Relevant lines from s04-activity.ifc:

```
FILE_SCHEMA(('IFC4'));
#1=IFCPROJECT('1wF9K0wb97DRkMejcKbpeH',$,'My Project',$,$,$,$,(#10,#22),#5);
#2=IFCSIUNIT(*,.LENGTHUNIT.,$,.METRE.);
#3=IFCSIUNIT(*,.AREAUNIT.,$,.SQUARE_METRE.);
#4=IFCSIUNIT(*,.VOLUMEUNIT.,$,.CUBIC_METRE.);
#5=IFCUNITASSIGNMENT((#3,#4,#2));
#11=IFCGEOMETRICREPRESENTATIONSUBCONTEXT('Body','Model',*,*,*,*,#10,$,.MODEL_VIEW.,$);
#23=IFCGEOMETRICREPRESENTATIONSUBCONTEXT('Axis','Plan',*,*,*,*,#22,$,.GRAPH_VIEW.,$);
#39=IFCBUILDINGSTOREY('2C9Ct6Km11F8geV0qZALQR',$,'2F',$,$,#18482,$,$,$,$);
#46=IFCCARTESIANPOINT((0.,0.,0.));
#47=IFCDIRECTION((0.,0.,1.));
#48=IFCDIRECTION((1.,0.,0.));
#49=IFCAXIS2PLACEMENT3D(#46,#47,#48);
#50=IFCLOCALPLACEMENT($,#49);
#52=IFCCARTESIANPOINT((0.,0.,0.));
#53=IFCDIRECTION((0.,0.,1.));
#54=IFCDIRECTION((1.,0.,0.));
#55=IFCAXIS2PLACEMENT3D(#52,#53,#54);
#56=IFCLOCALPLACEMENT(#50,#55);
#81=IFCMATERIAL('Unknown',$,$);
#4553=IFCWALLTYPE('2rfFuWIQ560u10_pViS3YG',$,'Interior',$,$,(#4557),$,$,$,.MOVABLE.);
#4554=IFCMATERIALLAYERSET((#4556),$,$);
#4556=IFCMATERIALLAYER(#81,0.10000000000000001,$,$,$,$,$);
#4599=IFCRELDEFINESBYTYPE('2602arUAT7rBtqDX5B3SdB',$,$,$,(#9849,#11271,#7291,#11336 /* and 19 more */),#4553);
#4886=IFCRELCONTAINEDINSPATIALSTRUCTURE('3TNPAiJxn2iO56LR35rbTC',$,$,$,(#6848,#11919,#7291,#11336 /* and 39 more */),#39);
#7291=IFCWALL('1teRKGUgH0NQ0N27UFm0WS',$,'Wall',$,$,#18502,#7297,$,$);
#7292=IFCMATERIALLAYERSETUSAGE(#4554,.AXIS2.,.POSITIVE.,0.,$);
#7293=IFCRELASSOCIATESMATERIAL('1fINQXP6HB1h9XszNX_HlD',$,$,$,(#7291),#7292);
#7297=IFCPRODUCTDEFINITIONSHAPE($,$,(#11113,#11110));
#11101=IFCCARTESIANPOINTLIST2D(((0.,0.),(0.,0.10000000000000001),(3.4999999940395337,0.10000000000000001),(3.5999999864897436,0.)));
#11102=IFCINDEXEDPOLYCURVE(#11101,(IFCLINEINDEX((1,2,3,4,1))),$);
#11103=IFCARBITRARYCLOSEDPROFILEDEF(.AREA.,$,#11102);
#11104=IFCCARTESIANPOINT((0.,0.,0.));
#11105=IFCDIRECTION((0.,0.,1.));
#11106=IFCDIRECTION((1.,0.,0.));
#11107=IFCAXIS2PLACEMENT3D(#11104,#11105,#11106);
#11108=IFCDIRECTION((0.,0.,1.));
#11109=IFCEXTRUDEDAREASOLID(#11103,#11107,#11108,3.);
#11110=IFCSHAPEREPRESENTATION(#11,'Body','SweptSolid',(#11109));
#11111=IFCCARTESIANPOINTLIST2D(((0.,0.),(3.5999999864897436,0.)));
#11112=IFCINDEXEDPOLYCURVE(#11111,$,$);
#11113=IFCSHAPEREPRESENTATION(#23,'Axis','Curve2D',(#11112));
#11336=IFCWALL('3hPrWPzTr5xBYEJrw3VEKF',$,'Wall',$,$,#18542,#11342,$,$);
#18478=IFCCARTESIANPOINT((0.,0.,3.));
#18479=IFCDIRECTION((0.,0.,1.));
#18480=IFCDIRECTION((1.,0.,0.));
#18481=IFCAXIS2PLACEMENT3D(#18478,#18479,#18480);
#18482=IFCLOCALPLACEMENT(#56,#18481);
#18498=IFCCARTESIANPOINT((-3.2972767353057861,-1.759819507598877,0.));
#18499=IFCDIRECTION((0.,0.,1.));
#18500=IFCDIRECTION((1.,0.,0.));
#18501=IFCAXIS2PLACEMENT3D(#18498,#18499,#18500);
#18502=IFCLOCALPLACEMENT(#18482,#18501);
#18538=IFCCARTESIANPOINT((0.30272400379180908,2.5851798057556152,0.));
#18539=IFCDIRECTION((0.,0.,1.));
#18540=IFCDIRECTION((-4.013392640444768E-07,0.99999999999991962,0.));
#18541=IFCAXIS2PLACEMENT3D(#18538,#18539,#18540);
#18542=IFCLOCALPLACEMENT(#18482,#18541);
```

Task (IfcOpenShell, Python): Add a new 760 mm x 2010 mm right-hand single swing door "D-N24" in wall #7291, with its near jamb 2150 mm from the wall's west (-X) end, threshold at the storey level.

```python
import numpy as np
import ifcopenshell
import ifcopenshell.api.feature
import ifcopenshell.api.geometry
import ifcopenshell.api.root
import ifcopenshell.api.spatial
import ifcopenshell.geom
import ifcopenshell.util.element
import ifcopenshell.util.placement
import ifcopenshell.util.representation
import ifcopenshell.util.shape
import ifcopenshell.util.unit

model = ifcopenshell.open("s04-activity.ifc")
unit_scale = ifcopenshell.util.unit.calculate_unit_scale(model)
settings = ifcopenshell.geom.settings()


def volume(element):
    """Net volume in cubic metres, openings subtracted."""
    shape = ifcopenshell.geom.create_shape(settings, element)
    return ifcopenshell.util.shape.get_volume(shape.geometry)


wall = model.by_guid("1teRKGUgH0NQ0N27UFm0WS")
storey = ifcopenshell.util.element.get_container(wall, ifc_class="IfcBuildingStorey")
context = ifcopenshell.util.representation.get_context(model, "Model", "Body", "MODEL_VIEW")
before = volume(wall)

width, height, from_end, sill = 0.76, 2.01, 2.15, 0.0  # metres

# The wall runs along its own X axis, and the end named is its -X end.
wall_shape = ifcopenshell.geom.create_shape(settings, wall)
x, y, z = ifcopenshell.util.shape.get_vertices(wall_shape.geometry).T
start = x.min() + from_end
face, thickness = float(y.min()), float(y.max() - y.min())
wall_matrix = ifcopenshell.util.placement.get_local_placement(wall.ObjectPlacement)
level = ifcopenshell.util.placement.get_local_placement(storey.ObjectPlacement)[2, 3]


def in_wall(x, y):
    """Placement at x, y metres in the wall's axes, at sill height."""
    matrix = wall_matrix.copy()
    matrix[:, 3] = wall_matrix @ np.array([x / unit_scale, y / unit_scale, 0.0, 1.0])
    matrix[2, 3] = level + sill / unit_scale
    return matrix


# Opening: a box that overshoots both wall faces by 50 mm.
opening = ifcopenshell.api.root.create_entity(model, ifc_class="IfcOpeningElement", predefined_type="OPENING")
box = ifcopenshell.api.geometry.add_wall_representation(
    model, context=context, length=width, height=height, thickness=thickness + 0.1
)
ifcopenshell.api.geometry.assign_representation(model, product=opening, representation=box)
ifcopenshell.api.geometry.edit_object_placement(model, product=opening, matrix=in_wall(start, face - 0.05), is_si=False)
ifcopenshell.api.feature.add_feature(model, feature=opening, element=wall)

door = ifcopenshell.api.root.create_entity(model, ifc_class="IfcDoor", name="D-N24", predefined_type="DOOR")
door.OverallWidth, door.OverallHeight = width / unit_scale, height / unit_scale
door.OperationType = "SINGLE_SWING_RIGHT"
body = ifcopenshell.api.geometry.add_door_representation(
    model,
    context=context,
    overall_width=door.OverallWidth,
    overall_height=door.OverallHeight,
    operation_type="SINGLE_SWING_RIGHT",
    lining_properties={"LiningDepth": thickness / unit_scale, "ThresholdDepth": thickness / unit_scale},
)
ifcopenshell.api.geometry.assign_representation(model, product=door, representation=body)
ifcopenshell.api.spatial.assign_container(model, products=[door], relating_structure=storey)
ifcopenshell.api.feature.add_filling(model, opening=opening, element=door)

# The lining spans the wall, so the door starts at the wall face.
ifcopenshell.api.geometry.edit_object_placement(model, product=door, matrix=in_wall(start, face), is_si=False)

after = volume(wall)

print(f"wall volume {before:.3f} -> {after:.3f} m3")

model.write("s04-activity_updated.ifc")
```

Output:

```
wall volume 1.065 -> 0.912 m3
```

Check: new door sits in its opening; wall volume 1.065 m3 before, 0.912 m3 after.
